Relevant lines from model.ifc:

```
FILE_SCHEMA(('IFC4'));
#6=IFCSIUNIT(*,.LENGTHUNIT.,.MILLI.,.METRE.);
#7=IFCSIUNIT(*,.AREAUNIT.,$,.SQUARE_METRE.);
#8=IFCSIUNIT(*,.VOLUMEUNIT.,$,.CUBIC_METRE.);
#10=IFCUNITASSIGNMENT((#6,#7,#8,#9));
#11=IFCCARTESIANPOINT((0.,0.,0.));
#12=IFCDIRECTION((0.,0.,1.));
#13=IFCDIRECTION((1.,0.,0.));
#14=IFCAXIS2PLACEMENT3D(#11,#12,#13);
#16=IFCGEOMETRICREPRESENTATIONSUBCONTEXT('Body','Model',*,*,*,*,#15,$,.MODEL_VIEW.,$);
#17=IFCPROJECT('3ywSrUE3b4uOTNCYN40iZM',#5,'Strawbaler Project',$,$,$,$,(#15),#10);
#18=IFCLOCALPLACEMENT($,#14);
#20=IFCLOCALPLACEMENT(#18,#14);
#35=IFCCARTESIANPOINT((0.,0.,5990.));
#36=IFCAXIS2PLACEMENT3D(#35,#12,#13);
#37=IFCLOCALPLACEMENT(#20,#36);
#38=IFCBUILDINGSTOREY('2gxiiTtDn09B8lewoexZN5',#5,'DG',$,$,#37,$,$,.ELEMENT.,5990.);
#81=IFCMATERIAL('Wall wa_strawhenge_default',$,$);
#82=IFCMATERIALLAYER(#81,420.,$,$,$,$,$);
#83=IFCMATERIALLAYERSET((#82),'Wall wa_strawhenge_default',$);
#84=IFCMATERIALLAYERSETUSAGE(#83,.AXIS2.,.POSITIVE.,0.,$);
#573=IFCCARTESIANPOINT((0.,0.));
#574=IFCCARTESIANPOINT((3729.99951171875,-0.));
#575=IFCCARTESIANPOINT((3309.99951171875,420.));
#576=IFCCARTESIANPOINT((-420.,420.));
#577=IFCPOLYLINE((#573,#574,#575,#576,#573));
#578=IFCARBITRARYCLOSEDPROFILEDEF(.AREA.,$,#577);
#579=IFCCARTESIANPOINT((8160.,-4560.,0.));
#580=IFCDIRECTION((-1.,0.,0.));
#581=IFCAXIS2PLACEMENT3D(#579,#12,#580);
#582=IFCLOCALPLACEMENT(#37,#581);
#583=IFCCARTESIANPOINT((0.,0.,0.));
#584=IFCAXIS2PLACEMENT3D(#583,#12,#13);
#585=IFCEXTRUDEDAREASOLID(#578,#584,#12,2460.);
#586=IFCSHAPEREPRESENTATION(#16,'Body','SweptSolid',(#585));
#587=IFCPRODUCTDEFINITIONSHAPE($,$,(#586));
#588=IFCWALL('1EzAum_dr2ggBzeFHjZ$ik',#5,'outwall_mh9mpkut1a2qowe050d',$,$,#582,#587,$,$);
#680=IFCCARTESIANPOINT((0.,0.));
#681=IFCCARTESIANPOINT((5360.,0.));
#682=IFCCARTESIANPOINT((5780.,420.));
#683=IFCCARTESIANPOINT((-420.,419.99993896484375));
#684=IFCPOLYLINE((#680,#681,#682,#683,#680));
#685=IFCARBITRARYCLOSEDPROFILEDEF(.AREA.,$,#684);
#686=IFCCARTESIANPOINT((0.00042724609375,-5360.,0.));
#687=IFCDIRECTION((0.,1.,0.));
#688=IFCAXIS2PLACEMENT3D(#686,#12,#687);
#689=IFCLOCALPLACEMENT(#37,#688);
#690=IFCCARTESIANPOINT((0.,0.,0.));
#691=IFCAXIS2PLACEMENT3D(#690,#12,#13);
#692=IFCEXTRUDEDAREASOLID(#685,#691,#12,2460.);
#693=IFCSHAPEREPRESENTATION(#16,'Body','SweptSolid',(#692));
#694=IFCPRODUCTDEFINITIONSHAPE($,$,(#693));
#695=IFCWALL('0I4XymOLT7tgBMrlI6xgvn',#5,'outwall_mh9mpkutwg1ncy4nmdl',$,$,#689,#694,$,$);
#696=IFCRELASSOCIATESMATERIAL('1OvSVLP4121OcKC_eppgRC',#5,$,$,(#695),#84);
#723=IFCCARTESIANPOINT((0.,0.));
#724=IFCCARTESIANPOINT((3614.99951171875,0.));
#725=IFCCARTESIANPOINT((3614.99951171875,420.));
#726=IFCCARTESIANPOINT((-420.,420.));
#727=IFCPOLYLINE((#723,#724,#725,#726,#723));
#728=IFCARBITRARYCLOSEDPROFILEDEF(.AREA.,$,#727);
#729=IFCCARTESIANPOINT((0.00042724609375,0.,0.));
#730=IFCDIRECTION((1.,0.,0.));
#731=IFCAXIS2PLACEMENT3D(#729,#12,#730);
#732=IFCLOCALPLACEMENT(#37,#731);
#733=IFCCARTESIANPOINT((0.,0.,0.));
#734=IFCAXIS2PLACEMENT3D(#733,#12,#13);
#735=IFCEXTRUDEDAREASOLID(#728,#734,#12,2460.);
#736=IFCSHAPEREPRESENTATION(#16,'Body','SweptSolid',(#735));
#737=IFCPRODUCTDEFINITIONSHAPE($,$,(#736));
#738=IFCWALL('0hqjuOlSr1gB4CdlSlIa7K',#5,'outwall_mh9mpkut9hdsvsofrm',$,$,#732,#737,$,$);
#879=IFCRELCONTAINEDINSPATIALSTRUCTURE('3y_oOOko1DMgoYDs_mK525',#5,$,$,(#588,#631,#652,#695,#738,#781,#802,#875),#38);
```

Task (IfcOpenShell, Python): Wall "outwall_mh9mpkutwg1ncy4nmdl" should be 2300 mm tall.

```python
import ifcopenshell
import ifcopenshell.geom
import ifcopenshell.util.representation
import ifcopenshell.util.shape
import ifcopenshell.util.unit

model = ifcopenshell.open("model.ifc")
unit_scale = ifcopenshell.util.unit.calculate_unit_scale(model)
settings = ifcopenshell.geom.settings()


def volume(element):
    """Net volume in cubic metres, openings subtracted."""
    shape = ifcopenshell.geom.create_shape(settings, element)
    return ifcopenshell.util.shape.get_volume(shape.geometry)


wall = model.by_id(695)
before = volume(wall)

body = ifcopenshell.util.representation.get_representation(wall, "Model", "Body")
solid = body.Items[0]
old_height = solid.Depth
solid.Depth = 2.3 / unit_scale
after = volume(wall)

print(f"height {old_height:g} -> {solid.Depth:g}, volume {before:.3f} -> {after:.3f} m3")

model.write("model_v2.ifc")
```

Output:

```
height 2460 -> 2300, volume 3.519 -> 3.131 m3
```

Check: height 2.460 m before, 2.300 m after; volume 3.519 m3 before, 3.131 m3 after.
